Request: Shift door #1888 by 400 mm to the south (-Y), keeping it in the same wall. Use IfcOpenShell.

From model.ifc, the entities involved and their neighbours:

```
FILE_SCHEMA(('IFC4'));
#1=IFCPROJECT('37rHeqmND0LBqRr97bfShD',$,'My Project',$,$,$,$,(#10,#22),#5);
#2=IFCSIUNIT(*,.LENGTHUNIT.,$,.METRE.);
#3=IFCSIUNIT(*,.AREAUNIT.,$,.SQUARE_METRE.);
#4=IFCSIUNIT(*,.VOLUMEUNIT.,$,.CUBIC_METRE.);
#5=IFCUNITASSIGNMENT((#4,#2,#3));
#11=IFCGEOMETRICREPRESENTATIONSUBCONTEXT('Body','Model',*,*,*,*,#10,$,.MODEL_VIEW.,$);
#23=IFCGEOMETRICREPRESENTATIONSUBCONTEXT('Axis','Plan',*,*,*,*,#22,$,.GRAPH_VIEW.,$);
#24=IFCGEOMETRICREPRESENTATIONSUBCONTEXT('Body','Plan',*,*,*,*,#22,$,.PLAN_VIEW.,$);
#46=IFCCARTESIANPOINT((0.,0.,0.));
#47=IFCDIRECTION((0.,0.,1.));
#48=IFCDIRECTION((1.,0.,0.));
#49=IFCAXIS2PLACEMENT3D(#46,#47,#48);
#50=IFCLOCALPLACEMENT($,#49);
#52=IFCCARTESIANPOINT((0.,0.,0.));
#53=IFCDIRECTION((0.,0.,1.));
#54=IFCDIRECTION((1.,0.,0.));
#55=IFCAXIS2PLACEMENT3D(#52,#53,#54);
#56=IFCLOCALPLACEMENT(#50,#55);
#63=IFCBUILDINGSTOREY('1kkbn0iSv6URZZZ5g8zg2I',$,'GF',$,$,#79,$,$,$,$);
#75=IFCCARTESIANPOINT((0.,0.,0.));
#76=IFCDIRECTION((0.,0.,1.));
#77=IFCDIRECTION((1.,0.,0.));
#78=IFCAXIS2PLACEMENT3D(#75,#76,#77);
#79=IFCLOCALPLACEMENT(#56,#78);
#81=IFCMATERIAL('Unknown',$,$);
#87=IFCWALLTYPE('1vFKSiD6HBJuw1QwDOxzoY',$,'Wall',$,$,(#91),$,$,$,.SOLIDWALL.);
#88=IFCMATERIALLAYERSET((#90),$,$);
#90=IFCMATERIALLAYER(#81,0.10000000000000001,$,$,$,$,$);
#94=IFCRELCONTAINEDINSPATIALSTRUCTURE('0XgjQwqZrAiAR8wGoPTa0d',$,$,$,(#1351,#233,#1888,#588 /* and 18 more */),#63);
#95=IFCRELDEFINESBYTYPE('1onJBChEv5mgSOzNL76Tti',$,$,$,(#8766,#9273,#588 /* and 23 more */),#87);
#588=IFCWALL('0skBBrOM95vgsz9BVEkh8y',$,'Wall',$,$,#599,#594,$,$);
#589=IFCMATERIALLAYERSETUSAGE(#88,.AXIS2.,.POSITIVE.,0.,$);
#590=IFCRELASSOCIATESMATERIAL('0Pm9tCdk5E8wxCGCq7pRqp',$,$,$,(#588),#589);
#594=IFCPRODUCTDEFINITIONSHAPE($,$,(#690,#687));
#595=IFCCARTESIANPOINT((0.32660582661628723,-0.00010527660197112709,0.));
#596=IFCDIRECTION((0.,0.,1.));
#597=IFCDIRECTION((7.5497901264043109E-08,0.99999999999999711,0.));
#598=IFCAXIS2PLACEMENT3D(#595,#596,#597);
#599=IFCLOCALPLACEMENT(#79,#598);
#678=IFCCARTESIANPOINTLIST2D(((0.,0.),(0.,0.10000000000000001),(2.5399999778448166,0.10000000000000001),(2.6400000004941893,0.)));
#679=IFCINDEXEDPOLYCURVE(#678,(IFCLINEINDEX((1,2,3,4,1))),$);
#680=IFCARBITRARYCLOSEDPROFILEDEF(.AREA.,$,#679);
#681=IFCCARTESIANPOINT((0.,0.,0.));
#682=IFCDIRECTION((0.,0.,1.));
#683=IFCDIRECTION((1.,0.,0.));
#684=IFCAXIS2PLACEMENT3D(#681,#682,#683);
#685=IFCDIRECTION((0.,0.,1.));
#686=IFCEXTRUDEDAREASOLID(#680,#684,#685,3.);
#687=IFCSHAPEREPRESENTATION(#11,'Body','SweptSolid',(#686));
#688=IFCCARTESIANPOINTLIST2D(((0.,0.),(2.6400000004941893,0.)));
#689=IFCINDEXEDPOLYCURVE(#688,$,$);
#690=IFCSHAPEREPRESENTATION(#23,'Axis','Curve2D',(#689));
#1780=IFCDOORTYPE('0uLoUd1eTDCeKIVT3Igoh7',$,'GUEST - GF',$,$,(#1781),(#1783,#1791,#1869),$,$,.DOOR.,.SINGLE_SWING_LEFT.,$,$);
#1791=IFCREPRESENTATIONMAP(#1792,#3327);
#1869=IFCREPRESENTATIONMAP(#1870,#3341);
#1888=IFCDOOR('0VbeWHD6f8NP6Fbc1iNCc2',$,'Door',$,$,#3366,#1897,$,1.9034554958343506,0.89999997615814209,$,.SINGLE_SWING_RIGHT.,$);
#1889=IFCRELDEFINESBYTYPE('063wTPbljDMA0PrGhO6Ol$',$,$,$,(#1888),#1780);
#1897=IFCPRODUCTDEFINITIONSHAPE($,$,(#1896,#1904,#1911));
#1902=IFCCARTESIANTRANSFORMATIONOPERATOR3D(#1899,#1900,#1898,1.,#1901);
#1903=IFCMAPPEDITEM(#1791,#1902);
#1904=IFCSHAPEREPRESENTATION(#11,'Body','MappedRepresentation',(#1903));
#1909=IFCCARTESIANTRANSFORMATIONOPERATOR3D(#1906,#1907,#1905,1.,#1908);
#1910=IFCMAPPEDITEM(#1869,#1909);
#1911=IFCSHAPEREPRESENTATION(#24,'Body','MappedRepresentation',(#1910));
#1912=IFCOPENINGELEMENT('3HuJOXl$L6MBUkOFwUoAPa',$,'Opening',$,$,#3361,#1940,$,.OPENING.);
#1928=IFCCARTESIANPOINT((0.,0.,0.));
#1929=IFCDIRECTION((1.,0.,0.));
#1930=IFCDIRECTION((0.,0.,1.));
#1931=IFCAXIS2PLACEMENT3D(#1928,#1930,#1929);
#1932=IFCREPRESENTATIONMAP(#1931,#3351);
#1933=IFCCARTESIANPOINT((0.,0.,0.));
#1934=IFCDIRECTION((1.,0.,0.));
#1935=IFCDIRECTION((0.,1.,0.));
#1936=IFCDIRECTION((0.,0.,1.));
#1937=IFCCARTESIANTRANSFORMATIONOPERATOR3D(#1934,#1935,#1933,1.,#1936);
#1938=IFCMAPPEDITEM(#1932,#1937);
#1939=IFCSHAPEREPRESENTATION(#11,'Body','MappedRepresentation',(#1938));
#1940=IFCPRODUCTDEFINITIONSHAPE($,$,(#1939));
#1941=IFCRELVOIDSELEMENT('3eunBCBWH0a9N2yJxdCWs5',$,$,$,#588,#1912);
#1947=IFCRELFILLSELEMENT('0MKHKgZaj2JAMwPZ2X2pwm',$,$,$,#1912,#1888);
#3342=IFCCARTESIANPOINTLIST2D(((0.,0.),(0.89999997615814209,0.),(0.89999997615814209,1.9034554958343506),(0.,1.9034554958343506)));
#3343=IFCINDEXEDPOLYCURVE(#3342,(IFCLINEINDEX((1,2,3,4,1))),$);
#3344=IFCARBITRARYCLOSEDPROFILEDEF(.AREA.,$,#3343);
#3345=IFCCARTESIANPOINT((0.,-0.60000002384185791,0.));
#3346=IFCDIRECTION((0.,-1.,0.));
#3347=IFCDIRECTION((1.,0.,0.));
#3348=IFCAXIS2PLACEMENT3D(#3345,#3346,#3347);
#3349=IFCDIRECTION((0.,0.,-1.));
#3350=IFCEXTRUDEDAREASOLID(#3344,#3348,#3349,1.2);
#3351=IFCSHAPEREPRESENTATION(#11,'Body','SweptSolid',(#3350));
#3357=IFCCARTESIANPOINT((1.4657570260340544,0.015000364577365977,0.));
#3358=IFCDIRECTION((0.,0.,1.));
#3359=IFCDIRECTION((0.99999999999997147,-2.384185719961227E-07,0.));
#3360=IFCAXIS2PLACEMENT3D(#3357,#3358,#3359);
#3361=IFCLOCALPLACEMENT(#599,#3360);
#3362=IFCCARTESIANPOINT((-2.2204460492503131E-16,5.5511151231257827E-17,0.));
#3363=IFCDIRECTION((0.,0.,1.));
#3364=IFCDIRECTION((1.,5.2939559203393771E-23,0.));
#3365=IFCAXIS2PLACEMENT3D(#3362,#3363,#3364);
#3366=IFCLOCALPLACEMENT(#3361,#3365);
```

```python
import ifcopenshell
import ifcopenshell.api.geometry
import ifcopenshell.util.placement

model = ifcopenshell.open("model.ifc")

door = model.by_id(1888)
opening = door.FillsVoids[0].RelatingOpeningElement
wall = opening.VoidsElements[0].RelatingBuildingElement

wall_matrix = ifcopenshell.util.placement.get_local_placement(wall.ObjectPlacement)
shift = wall_matrix[:3, 0] * -0.4
before = ifcopenshell.util.placement.get_local_placement(door.ObjectPlacement)[:3, 3].copy()

# The door is placed relative to its opening, so it follows when the opening moves.
matrix = ifcopenshell.util.placement.get_local_placement(opening.ObjectPlacement)
matrix[:3, 3] += shift
ifcopenshell.api.geometry.edit_object_placement(
    model, product=opening, matrix=matrix, is_si=False, should_transform_children=True
)

after = ifcopenshell.util.placement.get_local_placement(door.ObjectPlacement)[:3, 3]
print("door moved by", (after - before).round(3) + 0.0)

model.write("model_updated.ifc")
```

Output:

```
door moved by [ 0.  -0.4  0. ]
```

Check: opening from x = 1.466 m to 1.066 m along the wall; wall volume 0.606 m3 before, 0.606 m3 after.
